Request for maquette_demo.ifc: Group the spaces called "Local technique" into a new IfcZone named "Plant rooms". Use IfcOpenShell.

First a look at what the model holds.

```python
import ifcopenshell

model = ifcopenshell.open("maquette_demo.ifc")
print(model.schema)
seen = {}
for space in model.by_type("IfcSpace"):
    seen[space.LongName] = seen.get(space.LongName, 0) + 1
for name, count in sorted(seen.items(), key=str):
    print(count, "x", name)
print("zones:", [z.Name for z in model.by_type("IfcZone")][:20])
```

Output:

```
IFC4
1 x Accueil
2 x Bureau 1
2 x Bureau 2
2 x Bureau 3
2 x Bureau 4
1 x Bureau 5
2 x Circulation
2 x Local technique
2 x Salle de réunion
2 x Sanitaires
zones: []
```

```python
import ifcopenshell
import ifcopenshell.api.group
import ifcopenshell.api.root

model = ifcopenshell.open("maquette_demo.ifc")

names = {"Local technique"}
spaces = [s for s in model.by_type("IfcSpace") if s.LongName in names]

zone = ifcopenshell.api.root.create_entity(model, ifc_class="IfcZone", name="Plant rooms")
ifcopenshell.api.group.assign_group(model, products=spaces, group=zone)
print(len(spaces), "spaces in", zone.Name)

model.write("maquette_demo_updated.ifc")
```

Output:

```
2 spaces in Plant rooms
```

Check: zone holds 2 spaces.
